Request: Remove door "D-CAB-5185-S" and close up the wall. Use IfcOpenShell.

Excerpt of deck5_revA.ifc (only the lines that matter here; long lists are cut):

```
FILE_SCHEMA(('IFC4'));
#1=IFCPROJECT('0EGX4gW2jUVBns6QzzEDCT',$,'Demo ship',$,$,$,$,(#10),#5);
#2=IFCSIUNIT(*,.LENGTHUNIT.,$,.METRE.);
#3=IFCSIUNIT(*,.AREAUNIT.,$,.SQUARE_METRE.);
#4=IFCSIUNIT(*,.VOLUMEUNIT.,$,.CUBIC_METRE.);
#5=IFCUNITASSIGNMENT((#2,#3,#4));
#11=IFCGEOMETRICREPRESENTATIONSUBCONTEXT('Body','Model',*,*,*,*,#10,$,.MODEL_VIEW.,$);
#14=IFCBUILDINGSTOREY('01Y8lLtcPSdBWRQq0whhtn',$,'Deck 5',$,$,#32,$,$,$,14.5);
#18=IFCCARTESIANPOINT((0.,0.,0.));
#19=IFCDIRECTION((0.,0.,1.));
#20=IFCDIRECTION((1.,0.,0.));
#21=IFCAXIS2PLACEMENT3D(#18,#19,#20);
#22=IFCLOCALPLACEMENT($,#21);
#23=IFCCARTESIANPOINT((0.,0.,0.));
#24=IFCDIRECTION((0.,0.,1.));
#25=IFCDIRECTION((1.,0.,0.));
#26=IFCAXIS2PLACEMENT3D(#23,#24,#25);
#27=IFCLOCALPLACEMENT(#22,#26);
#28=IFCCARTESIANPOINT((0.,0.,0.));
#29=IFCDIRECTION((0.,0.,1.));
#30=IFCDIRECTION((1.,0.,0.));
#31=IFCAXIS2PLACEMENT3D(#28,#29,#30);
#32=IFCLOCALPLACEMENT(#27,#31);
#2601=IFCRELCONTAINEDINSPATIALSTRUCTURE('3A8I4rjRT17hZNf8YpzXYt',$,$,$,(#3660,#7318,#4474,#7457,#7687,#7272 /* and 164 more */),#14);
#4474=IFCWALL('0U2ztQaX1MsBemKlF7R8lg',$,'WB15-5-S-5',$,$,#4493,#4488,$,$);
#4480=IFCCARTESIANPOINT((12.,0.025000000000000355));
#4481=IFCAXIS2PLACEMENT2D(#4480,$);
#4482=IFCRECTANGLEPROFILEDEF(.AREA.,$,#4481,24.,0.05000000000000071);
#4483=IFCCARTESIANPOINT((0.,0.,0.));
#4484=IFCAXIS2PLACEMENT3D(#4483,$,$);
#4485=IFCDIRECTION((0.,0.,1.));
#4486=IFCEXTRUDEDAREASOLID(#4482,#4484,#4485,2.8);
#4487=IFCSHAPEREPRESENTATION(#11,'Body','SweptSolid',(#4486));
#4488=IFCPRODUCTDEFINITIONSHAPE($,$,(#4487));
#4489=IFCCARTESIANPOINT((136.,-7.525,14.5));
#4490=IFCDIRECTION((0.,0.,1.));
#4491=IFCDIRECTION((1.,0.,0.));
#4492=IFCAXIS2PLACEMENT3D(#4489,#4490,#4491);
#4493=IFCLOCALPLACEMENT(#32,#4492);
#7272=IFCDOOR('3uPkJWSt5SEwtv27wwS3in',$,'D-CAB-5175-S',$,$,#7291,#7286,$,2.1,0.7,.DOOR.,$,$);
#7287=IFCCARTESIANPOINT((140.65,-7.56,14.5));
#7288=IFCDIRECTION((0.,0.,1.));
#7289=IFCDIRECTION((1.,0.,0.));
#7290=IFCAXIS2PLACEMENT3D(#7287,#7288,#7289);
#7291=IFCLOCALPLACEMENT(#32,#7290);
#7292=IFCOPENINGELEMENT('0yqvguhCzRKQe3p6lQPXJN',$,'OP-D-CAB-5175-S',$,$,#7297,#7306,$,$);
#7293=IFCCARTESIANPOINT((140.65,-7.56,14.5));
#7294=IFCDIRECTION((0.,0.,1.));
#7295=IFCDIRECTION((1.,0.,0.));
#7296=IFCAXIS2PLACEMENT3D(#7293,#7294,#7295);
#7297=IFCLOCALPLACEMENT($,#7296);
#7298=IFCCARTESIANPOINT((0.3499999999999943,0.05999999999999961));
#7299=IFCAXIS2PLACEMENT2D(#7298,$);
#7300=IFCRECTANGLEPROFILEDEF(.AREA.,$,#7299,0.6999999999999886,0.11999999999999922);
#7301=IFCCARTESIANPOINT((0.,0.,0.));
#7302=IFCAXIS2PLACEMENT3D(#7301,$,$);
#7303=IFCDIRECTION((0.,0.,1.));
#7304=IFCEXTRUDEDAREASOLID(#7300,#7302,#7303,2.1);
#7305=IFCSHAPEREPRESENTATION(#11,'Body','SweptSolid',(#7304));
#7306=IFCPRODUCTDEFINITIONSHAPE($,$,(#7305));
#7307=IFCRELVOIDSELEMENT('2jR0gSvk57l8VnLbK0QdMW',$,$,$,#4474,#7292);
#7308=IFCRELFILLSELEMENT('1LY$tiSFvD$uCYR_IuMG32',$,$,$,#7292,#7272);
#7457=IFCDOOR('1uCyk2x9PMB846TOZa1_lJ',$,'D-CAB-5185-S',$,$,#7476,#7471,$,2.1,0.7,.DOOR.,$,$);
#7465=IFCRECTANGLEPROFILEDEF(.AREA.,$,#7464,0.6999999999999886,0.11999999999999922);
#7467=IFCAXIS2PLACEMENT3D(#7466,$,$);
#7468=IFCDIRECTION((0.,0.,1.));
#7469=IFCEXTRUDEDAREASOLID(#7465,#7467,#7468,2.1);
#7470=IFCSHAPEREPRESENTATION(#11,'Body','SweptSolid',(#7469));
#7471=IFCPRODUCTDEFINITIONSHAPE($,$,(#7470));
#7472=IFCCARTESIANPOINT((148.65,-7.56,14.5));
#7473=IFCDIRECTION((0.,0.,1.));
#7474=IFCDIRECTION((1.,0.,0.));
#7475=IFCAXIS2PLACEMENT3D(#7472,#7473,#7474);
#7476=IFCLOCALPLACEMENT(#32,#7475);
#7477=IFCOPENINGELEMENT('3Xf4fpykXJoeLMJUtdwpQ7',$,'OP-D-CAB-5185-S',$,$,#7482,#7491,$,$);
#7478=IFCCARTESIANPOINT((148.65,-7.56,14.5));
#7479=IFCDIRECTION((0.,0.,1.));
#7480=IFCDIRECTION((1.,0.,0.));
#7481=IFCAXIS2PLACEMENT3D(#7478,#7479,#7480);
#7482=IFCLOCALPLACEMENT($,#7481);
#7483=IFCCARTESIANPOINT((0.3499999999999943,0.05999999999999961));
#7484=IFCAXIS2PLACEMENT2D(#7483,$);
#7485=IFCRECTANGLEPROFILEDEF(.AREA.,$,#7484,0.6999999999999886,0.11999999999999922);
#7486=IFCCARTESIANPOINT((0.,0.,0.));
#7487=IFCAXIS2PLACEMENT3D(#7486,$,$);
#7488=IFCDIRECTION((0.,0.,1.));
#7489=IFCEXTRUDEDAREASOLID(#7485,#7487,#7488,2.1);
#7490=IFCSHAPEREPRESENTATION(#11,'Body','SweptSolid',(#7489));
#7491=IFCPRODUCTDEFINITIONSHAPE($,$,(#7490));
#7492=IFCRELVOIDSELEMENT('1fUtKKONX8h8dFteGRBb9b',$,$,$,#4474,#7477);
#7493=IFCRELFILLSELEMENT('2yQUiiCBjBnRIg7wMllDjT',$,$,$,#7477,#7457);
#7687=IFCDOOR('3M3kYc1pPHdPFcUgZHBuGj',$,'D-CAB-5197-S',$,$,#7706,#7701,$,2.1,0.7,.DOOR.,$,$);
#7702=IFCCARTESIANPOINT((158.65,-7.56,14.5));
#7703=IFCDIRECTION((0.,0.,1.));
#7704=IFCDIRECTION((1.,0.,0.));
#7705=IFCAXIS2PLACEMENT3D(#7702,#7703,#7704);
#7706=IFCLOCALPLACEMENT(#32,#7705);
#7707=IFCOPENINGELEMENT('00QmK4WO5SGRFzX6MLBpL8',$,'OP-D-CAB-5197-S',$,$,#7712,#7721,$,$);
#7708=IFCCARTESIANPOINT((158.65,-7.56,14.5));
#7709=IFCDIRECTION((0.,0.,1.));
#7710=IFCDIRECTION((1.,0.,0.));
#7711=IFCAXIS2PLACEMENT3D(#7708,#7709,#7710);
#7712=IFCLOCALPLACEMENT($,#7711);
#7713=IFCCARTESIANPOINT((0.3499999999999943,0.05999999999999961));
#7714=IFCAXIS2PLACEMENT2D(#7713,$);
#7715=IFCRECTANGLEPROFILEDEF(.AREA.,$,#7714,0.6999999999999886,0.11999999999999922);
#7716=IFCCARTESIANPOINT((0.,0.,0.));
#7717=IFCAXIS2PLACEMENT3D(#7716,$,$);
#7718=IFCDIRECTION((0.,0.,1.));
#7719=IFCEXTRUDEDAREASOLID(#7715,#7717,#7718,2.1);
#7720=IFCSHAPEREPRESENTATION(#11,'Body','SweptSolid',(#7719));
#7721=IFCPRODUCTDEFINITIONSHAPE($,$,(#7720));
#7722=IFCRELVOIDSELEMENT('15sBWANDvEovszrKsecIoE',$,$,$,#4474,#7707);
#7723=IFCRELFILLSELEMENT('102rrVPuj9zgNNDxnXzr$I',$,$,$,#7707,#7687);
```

```python
import ifcopenshell
import ifcopenshell.api.feature
import ifcopenshell.api.root
import ifcopenshell.geom
import ifcopenshell.util.shape

model = ifcopenshell.open("deck5_revA.ifc")
settings = ifcopenshell.geom.settings()


def volume(element):
    """Net volume in cubic metres, openings subtracted."""
    shape = ifcopenshell.geom.create_shape(settings, element)
    return ifcopenshell.util.shape.get_volume(shape.geometry)


door = model.by_id(7457)
opening = door.FillsVoids[0].RelatingOpeningElement
wall = opening.VoidsElements[0].RelatingBuildingElement
before = volume(wall)

ifcopenshell.api.root.remove_product(model, product=door)
ifcopenshell.api.feature.remove_feature(model, feature=opening)

after = volume(wall)

print(f"wall volume {before:.3f} -> {after:.3f} m3")

model.write("deck5_revA-out.ifc")
```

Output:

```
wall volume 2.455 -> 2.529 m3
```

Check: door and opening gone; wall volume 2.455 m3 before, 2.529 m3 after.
